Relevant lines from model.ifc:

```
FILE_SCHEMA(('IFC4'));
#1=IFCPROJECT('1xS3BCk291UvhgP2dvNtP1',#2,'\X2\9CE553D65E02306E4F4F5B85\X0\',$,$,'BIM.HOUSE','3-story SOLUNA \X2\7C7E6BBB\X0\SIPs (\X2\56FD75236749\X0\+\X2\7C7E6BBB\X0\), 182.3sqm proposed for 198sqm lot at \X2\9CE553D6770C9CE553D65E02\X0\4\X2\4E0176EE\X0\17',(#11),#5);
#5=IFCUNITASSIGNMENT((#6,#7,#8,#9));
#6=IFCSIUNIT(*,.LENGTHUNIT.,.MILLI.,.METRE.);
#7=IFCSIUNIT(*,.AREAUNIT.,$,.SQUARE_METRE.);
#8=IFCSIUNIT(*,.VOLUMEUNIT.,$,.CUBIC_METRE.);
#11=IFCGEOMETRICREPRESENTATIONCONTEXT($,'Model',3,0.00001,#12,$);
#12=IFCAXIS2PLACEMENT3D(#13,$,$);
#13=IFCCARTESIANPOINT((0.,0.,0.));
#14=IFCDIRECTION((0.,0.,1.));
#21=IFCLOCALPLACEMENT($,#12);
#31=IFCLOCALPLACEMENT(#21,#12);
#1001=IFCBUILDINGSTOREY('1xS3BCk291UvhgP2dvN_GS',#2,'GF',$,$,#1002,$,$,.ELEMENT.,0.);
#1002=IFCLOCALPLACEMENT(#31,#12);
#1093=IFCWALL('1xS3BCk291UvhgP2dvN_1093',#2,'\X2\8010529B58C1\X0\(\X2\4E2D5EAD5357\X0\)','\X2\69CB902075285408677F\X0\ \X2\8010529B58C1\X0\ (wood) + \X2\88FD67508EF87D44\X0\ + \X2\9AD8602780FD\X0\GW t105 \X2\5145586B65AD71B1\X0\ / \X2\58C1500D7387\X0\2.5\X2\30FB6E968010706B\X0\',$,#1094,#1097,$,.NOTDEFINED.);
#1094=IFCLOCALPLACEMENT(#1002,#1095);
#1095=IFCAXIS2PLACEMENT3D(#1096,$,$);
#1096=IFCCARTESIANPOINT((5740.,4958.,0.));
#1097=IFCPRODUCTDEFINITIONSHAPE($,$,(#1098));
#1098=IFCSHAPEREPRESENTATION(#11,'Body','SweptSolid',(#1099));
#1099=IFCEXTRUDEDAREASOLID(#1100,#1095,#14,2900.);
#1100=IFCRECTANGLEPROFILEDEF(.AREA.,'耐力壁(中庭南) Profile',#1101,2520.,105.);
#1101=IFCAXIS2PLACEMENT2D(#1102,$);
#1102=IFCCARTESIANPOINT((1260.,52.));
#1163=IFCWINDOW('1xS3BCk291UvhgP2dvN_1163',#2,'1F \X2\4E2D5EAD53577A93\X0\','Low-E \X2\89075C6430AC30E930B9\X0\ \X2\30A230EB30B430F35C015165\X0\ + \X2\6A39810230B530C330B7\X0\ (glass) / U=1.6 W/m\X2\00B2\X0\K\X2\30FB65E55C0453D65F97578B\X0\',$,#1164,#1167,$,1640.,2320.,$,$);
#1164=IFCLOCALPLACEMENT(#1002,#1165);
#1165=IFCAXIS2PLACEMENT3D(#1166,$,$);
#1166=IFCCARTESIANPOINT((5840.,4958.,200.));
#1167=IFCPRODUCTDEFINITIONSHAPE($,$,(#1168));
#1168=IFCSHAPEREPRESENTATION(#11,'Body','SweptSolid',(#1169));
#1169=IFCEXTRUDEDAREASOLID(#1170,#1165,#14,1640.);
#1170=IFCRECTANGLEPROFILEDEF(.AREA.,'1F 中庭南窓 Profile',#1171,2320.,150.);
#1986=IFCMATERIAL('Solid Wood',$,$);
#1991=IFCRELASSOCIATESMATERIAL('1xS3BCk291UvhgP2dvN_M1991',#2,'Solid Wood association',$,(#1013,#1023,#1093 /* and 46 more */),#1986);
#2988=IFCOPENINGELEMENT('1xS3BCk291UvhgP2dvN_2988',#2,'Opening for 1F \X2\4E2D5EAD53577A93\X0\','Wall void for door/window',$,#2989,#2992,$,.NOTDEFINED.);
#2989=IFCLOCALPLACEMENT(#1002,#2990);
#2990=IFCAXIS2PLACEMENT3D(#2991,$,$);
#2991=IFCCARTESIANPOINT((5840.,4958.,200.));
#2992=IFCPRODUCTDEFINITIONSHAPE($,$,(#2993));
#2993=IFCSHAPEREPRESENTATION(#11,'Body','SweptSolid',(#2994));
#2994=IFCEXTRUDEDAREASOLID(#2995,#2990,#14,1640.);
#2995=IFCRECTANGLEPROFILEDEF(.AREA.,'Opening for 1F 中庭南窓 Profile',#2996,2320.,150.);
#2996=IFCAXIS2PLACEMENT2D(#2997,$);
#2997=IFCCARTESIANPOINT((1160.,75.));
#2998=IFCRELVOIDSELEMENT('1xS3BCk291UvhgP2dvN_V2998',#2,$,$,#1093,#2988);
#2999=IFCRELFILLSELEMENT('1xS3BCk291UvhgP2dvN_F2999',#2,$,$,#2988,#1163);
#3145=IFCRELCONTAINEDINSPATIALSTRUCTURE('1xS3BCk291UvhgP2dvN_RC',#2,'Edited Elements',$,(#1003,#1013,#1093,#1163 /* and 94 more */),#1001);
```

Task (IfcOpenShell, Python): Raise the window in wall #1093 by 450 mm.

```python
import numpy as np
import ifcopenshell
import ifcopenshell.api.geometry
import ifcopenshell.util.placement
import ifcopenshell.util.unit

model = ifcopenshell.open("model.ifc")
unit_scale = ifcopenshell.util.unit.calculate_unit_scale(model)

window = model.by_guid("1xS3BCk291UvhgP2dvN_1163")
opening = window.FillsVoids[0].RelatingOpeningElement
dz = 450.0

shift = np.array([0.0, 0.0, dz])
# The window is not placed relative to its opening, so move both.
for product in (opening, window):
    matrix = ifcopenshell.util.placement.get_local_placement(product.ObjectPlacement)
    matrix[:3, 3] += shift
    ifcopenshell.api.geometry.edit_object_placement(model, product=product, matrix=matrix, is_si=False)

print(f"moved by {dz * unit_scale:+.3f} m")

model.write("model_v2.ifc")
```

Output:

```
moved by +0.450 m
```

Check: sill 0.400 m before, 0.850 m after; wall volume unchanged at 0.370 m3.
